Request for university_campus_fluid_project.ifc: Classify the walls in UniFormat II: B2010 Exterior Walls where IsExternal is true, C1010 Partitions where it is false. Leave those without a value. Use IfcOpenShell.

First a look at what the model holds.

```python
import ifcopenshell
import ifcopenshell.util.element

model = ifcopenshell.open("university_campus_fluid_project.ifc")
print(model.schema)
print("classifications:", [c.Name for c in model.by_type("IfcClassification")])
values = [ifcopenshell.util.element.get_pset(e, "Pset_WallCommon", "IsExternal") for e in model.by_type("IfcWall")]
for value in (True, False, None):
    print("IsExternal", value, values.count(value))
```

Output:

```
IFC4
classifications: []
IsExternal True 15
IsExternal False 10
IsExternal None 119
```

```python
import ifcopenshell
import ifcopenshell.api.classification
import ifcopenshell.util.element

model = ifcopenshell.open("university_campus_fluid_project.ifc")

system = ifcopenshell.api.classification.add_classification(model, classification="UniFormat II")

walls = model.by_type("IfcWall")
external = {e: ifcopenshell.util.element.get_pset(e, "Pset_WallCommon", "IsExternal") for e in walls}
for flag, code, name in ((True, "B2010", "Exterior Walls"), (False, "C1010", "Partitions")):
    products = [e for e in walls if external[e] is flag]
    ifcopenshell.api.classification.add_reference(
        model, products=products, classification=system, identification=code, name=name
    )
    print(code, len(products))

model.write("university_campus_fluid_project-out.ifc")
```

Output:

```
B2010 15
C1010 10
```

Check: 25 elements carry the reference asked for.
